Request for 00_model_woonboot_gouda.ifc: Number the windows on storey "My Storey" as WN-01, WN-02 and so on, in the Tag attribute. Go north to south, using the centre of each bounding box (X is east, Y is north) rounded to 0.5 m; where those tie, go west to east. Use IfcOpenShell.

First a look at what the model holds.

```python
import ifcopenshell
import ifcopenshell.util.element
import ifcopenshell.util.placement

model = ifcopenshell.open("00_model_woonboot_gouda.ifc")
print(model.schema)
storey = next(s for s in model.by_type("IfcBuildingStorey") if s.Name == "My Storey")
windows = [e for e in ifcopenshell.util.element.get_decomposition(storey) if e.is_a("IfcWindow")]
for e in sorted(windows, key=lambda e: e.id()):
    origin = ifcopenshell.util.placement.get_local_placement(e.ObjectPlacement)[:3, 3]
    print(e.id(), e.Tag, e.Name, origin.round(2) + 0.0, sep=" | ")
```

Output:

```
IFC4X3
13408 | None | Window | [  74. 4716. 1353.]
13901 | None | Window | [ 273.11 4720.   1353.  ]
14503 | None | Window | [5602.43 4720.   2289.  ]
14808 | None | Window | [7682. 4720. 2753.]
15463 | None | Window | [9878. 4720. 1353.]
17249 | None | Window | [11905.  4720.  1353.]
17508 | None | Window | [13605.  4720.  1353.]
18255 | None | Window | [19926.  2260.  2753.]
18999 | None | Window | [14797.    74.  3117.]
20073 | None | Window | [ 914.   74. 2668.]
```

```python
import ifcopenshell
import ifcopenshell.geom
import ifcopenshell.util.element
import ifcopenshell.util.shape

model = ifcopenshell.open("00_model_woonboot_gouda.ifc")
settings = ifcopenshell.geom.settings()
settings.set("use-world-coords", True)


def centre(element):
    shape = ifcopenshell.geom.create_shape(settings, element)
    return ifcopenshell.util.shape.get_bbox_centroid(shape.geometry)


storey = next(s for s in model.by_type("IfcBuildingStorey") if s.Name == "My Storey")
windows = [e for e in ifcopenshell.util.element.get_decomposition(storey) if e.is_a("IfcWindow")]

# Insertion points can sit at a corner or the storey origin, so sort by the geometry (in metres).
centres = {e: centre(e) for e in windows}
windows.sort(key=lambda e: (-round(centres[e][1] / 0.5), centres[e][0]))

for i, e in enumerate(windows, start=1):
    number = f"WN-{i:02d}"
    e.Tag = number
    print(e.id(), number)

model.write("00_model_woonboot_gouda_v2.ifc")
```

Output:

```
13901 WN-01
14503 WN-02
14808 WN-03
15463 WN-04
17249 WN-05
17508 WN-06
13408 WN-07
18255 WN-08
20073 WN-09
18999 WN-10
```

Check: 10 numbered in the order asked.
